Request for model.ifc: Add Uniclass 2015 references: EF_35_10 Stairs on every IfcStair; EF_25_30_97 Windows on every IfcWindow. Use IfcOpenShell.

First a look at what the model holds.

```python
import ifcopenshell

model = ifcopenshell.open("model.ifc")
print(model.schema)
print("classifications:", [c.Name for c in model.by_type("IfcClassification")])
for ifc_class in ("IfcDoor", "IfcRoof", "IfcStair", "IfcWall", "IfcWindow"):
    print(ifc_class, len(model.by_type(ifc_class)))
```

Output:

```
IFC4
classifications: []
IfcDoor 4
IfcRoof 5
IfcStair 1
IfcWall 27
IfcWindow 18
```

```python
import ifcopenshell
import ifcopenshell.api.classification

model = ifcopenshell.open("model.ifc")

system = ifcopenshell.api.classification.add_classification(model, classification="Uniclass 2015")

codes = {
    "IfcStair": ("EF_35_10", "Stairs"),
    "IfcWindow": ("EF_25_30_97", "Windows"),
}
for ifc_class, (code, name) in codes.items():
    products = model.by_type(ifc_class)
    ifcopenshell.api.classification.add_reference(
        model, products=products, classification=system, identification=code, name=name
    )
    print(code, len(products))

model.write("model_edited.ifc")
```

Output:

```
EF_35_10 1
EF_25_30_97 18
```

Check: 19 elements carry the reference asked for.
